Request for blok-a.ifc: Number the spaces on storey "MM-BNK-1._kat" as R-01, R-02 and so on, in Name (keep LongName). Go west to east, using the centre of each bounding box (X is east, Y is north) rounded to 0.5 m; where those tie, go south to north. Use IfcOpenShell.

First a look at what the model holds.

```python
import ifcopenshell
import ifcopenshell.util.element
import ifcopenshell.util.placement

model = ifcopenshell.open("blok-a.ifc")
print(model.schema)
storey = next(s for s in model.by_type("IfcBuildingStorey") if s.Name == "MM-BNK-1._kat")
spaces = [e for e in ifcopenshell.util.element.get_decomposition(storey) if e.is_a("IfcSpace")]
for e in sorted(spaces, key=lambda e: e.id()):
    origin = ifcopenshell.util.placement.get_local_placement(e.ObjectPlacement)[:3, 3]
    print(e.id(), e.Name, e.LongName, origin.round(2) + 0.0, sep=" | ")
```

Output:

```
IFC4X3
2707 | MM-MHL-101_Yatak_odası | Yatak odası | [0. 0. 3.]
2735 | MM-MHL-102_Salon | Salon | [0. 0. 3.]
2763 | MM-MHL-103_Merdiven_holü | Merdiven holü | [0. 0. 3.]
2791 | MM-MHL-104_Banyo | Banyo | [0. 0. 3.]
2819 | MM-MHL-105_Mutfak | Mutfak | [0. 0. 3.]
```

```python
import ifcopenshell
import ifcopenshell.geom
import ifcopenshell.util.element
import ifcopenshell.util.shape

model = ifcopenshell.open("blok-a.ifc")
settings = ifcopenshell.geom.settings()
settings.set("use-world-coords", True)


def centre(element):
    shape = ifcopenshell.geom.create_shape(settings, element)
    return ifcopenshell.util.shape.get_bbox_centroid(shape.geometry)


storey = next(s for s in model.by_type("IfcBuildingStorey") if s.Name == "MM-BNK-1._kat")
spaces = [e for e in ifcopenshell.util.element.get_decomposition(storey) if e.is_a("IfcSpace")]

# Insertion points can sit at a corner or the storey origin, so sort by the geometry (in metres).
centres = {e: centre(e) for e in spaces}
spaces.sort(key=lambda e: (round(centres[e][0] / 0.5), centres[e][1]))

for i, e in enumerate(spaces, start=1):
    number = f"R-{i:02d}"
    e.Name = number
    print(e.id(), number)

model.write("blok-a_edited.ifc")
```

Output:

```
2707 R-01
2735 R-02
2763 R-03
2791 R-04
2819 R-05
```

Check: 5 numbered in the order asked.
